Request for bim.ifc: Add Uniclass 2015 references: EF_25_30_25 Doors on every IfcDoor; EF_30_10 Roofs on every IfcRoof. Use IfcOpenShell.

First a look at what the model holds.

```python
import ifcopenshell

model = ifcopenshell.open("bim.ifc")
print(model.schema)
print("classifications:", [c.Name for c in model.by_type("IfcClassification")])
for ifc_class in ("IfcDoor", "IfcRoof", "IfcStair", "IfcWall", "IfcWindow"):
    print(ifc_class, len(model.by_type(ifc_class)))
```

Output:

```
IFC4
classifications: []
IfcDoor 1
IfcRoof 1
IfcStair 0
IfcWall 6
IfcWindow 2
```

```python
import ifcopenshell
import ifcopenshell.api.classification

model = ifcopenshell.open("bim.ifc")

system = ifcopenshell.api.classification.add_classification(model, classification="Uniclass 2015")

codes = {
    "IfcDoor": ("EF_25_30_25", "Doors"),
    "IfcRoof": ("EF_30_10", "Roofs"),
}
for ifc_class, (code, name) in codes.items():
    products = model.by_type(ifc_class)
    ifcopenshell.api.classification.add_reference(
        model, products=products, classification=system, identification=code, name=name
    )
    print(code, len(products))

model.write("bim_updated.ifc")
```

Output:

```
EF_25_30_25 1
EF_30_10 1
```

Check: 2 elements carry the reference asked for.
